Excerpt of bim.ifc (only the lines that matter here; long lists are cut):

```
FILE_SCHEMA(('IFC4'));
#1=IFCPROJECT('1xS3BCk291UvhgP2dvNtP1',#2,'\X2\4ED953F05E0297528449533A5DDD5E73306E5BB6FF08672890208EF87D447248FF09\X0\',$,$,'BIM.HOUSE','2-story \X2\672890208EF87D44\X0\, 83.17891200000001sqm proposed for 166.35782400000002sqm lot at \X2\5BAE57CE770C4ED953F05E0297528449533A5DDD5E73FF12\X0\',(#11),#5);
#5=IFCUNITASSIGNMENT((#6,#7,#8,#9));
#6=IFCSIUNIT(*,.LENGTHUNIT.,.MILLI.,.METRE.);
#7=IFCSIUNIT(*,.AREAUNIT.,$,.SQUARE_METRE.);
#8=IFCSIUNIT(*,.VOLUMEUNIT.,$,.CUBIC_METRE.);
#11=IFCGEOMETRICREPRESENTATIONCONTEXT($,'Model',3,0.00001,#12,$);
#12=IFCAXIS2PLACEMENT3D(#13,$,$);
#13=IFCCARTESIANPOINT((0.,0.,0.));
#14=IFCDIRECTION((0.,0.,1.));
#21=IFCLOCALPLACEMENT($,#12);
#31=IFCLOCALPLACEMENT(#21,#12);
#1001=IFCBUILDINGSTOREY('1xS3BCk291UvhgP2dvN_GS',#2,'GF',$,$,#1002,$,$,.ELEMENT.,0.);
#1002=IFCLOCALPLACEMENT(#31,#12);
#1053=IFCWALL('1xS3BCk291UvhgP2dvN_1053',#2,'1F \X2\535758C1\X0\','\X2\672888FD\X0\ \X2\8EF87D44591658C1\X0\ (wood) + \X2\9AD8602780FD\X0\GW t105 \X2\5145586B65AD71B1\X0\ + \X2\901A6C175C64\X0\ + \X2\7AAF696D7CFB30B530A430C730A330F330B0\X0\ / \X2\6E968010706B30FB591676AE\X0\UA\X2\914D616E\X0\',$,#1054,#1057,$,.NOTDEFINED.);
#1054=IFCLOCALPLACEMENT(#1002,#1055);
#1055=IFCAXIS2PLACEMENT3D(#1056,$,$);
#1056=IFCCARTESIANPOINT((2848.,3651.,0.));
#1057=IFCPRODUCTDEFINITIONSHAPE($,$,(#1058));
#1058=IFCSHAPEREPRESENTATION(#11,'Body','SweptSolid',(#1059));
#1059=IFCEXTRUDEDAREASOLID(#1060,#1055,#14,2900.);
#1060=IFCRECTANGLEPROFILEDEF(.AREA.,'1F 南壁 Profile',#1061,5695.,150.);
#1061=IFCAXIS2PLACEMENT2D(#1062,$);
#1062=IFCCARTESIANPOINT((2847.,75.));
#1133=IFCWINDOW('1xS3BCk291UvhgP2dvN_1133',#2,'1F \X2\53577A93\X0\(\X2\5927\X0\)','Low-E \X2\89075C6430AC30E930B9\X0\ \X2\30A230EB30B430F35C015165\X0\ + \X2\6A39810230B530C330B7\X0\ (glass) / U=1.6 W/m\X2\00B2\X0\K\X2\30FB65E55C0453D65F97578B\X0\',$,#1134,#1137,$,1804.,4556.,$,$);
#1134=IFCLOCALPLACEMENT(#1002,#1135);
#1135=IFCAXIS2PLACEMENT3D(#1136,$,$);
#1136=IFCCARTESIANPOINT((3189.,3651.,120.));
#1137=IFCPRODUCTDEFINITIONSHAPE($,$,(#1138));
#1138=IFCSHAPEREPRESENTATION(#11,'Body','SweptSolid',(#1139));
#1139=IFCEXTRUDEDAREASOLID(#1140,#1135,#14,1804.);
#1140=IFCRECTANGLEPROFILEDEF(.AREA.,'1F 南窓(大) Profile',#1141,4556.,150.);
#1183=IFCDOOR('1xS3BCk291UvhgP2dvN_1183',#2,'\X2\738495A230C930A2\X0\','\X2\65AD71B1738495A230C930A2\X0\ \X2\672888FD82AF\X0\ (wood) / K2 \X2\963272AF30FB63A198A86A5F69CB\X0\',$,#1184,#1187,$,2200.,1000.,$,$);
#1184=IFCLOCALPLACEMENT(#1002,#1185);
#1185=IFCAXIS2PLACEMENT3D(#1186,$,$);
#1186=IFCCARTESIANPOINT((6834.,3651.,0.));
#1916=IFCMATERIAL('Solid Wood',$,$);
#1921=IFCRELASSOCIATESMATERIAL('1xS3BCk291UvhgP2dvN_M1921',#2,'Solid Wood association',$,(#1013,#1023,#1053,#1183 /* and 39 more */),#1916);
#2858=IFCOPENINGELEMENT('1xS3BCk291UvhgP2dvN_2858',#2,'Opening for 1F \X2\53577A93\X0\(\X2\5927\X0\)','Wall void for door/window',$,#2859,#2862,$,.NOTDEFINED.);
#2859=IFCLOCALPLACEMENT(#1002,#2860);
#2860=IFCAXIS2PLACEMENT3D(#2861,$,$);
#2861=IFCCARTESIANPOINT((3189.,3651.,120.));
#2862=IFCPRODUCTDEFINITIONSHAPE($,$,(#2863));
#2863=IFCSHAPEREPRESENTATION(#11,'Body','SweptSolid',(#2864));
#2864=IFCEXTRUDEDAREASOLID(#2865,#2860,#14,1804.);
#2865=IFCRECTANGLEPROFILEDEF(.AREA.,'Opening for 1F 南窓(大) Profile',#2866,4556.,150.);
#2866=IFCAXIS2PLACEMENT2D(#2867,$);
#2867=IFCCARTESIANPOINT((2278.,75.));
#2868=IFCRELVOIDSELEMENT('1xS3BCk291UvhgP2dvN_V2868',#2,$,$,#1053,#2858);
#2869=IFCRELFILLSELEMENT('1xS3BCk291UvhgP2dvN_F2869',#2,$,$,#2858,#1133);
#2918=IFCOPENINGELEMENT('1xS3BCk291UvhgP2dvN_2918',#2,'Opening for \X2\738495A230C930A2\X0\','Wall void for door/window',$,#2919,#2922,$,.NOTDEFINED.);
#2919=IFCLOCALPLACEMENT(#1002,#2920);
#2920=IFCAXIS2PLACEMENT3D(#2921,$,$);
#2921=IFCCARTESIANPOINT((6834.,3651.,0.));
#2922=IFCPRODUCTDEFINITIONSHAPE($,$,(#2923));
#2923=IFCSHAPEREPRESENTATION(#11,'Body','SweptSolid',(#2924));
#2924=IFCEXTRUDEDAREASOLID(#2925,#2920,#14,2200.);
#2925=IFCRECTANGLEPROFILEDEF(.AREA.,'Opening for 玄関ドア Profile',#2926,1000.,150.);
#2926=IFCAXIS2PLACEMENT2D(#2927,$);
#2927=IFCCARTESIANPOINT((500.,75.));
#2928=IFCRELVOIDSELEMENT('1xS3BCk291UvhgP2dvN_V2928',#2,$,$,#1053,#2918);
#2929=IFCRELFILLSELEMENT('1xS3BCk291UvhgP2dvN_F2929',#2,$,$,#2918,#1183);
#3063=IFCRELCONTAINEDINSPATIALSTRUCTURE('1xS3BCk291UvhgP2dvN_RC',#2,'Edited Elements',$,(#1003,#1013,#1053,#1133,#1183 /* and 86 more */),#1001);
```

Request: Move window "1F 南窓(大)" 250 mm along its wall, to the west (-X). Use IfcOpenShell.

```python
import ifcopenshell
import ifcopenshell.api.geometry
import ifcopenshell.util.placement
import ifcopenshell.util.unit

model = ifcopenshell.open("bim.ifc")
unit_scale = ifcopenshell.util.unit.calculate_unit_scale(model)

window = model.by_guid("1xS3BCk291UvhgP2dvN_1133")
opening = window.FillsVoids[0].RelatingOpeningElement
wall = opening.VoidsElements[0].RelatingBuildingElement

wall_matrix = ifcopenshell.util.placement.get_local_placement(wall.ObjectPlacement)
shift = wall_matrix[:3, 0] * -0.25 / unit_scale
before = ifcopenshell.util.placement.get_local_placement(window.ObjectPlacement)[:3, 3].copy()

# The window is not placed relative to its opening, so move both.
for product in (opening, window):
    matrix = ifcopenshell.util.placement.get_local_placement(product.ObjectPlacement)
    matrix[:3, 3] += shift
    ifcopenshell.api.geometry.edit_object_placement(model, product=product, matrix=matrix, is_si=False)

after = ifcopenshell.util.placement.get_local_placement(window.ObjectPlacement)[:3, 3]
print("window moved by", (after - before).round(3) + 0.0)

model.write("bim-out.ifc")
```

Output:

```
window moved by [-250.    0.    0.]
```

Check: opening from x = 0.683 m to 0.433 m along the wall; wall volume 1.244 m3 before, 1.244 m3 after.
